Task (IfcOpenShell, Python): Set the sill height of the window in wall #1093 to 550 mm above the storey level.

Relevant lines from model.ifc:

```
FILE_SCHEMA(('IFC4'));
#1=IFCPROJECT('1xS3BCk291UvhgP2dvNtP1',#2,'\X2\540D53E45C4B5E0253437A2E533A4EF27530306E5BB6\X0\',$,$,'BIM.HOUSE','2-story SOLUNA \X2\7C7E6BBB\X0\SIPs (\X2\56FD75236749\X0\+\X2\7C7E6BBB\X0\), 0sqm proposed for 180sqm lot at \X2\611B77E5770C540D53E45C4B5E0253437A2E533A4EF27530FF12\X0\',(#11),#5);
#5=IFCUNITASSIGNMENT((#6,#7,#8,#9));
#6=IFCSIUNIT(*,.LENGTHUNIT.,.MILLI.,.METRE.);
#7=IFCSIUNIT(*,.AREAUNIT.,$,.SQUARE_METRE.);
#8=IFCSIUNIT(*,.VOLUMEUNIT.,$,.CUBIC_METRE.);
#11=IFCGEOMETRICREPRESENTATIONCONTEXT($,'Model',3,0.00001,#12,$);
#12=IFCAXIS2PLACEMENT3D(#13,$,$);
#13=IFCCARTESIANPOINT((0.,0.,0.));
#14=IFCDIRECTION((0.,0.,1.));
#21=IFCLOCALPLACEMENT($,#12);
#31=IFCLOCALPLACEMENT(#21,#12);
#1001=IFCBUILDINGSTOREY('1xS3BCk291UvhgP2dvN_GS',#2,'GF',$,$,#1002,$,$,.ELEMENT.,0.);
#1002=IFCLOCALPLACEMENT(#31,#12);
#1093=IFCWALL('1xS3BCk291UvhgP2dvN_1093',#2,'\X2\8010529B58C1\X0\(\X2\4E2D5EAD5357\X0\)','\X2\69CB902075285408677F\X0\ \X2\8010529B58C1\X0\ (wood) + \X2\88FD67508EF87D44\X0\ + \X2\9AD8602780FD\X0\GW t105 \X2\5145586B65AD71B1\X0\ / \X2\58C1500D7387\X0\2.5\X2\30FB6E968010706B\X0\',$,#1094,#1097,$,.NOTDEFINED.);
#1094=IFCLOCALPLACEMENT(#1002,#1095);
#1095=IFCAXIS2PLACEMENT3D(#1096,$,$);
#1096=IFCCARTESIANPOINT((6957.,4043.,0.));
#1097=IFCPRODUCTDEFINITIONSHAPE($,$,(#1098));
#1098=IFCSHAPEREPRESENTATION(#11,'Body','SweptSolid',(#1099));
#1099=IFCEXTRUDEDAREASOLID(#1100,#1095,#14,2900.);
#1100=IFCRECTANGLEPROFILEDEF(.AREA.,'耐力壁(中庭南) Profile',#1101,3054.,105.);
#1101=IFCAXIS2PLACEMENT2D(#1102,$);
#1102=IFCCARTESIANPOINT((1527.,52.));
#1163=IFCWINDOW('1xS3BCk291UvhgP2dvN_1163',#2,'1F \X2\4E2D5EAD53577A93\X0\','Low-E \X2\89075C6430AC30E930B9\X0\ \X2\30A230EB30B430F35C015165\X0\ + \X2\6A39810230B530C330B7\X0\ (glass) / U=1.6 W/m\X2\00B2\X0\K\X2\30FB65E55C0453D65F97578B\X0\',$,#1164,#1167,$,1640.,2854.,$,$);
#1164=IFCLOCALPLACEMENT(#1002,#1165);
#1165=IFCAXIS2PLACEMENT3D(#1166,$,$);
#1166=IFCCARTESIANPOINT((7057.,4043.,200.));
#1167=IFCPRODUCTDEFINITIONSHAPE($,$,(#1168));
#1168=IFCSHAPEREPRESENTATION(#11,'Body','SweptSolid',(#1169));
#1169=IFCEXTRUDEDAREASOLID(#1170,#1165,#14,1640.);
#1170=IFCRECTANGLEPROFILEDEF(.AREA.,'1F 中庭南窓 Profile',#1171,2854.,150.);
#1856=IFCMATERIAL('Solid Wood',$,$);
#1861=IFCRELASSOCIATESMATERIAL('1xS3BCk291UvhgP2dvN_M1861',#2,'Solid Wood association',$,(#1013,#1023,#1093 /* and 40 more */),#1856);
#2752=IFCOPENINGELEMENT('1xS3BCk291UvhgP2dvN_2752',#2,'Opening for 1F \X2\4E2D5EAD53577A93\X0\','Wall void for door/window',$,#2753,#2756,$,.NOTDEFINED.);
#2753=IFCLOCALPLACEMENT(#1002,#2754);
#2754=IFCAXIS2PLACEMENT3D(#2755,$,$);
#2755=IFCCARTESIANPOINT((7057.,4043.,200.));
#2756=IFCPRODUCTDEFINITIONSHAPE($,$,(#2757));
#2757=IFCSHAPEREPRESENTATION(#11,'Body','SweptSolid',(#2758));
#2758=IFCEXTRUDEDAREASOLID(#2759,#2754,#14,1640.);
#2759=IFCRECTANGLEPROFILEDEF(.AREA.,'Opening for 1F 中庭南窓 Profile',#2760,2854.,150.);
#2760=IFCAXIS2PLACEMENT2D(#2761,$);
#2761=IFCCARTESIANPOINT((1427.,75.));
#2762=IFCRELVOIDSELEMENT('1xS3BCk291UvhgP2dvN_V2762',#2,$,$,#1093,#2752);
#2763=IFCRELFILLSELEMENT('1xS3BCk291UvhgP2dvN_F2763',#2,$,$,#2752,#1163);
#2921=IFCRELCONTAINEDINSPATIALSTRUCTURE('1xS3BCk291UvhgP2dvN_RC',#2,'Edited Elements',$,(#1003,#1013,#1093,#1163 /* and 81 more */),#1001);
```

```python
import numpy as np
import ifcopenshell
import ifcopenshell.api.geometry
import ifcopenshell.geom
import ifcopenshell.util.element
import ifcopenshell.util.placement
import ifcopenshell.util.shape
import ifcopenshell.util.unit

model = ifcopenshell.open("model.ifc")
unit_scale = ifcopenshell.util.unit.calculate_unit_scale(model)

window = model.by_guid("1xS3BCk291UvhgP2dvN_1163")
opening = window.FillsVoids[0].RelatingOpeningElement
storey = ifcopenshell.util.element.get_container(window, ifc_class="IfcBuildingStorey")
level = ifcopenshell.util.placement.get_local_placement(storey.ObjectPlacement)[2, 3]

# The opening's origin need not be at the sill, so measure its lowest point.
shape = ifcopenshell.geom.create_shape(ifcopenshell.geom.settings(), opening)
bottom = ifcopenshell.util.shape.get_shape_bottom_elevation(shape, shape.geometry) / unit_scale
dz = level + 0.55 / unit_scale - bottom

shift = np.array([0.0, 0.0, dz])
# The window is not placed relative to its opening, so move both.
for product in (opening, window):
    matrix = ifcopenshell.util.placement.get_local_placement(product.ObjectPlacement)
    matrix[:3, 3] += shift
    ifcopenshell.api.geometry.edit_object_placement(model, product=product, matrix=matrix, is_si=False)

print(f"moved by {dz * unit_scale:+.3f} m")

model.write("model_rev.ifc")
```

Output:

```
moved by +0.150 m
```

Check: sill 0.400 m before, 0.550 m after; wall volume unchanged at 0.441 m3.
